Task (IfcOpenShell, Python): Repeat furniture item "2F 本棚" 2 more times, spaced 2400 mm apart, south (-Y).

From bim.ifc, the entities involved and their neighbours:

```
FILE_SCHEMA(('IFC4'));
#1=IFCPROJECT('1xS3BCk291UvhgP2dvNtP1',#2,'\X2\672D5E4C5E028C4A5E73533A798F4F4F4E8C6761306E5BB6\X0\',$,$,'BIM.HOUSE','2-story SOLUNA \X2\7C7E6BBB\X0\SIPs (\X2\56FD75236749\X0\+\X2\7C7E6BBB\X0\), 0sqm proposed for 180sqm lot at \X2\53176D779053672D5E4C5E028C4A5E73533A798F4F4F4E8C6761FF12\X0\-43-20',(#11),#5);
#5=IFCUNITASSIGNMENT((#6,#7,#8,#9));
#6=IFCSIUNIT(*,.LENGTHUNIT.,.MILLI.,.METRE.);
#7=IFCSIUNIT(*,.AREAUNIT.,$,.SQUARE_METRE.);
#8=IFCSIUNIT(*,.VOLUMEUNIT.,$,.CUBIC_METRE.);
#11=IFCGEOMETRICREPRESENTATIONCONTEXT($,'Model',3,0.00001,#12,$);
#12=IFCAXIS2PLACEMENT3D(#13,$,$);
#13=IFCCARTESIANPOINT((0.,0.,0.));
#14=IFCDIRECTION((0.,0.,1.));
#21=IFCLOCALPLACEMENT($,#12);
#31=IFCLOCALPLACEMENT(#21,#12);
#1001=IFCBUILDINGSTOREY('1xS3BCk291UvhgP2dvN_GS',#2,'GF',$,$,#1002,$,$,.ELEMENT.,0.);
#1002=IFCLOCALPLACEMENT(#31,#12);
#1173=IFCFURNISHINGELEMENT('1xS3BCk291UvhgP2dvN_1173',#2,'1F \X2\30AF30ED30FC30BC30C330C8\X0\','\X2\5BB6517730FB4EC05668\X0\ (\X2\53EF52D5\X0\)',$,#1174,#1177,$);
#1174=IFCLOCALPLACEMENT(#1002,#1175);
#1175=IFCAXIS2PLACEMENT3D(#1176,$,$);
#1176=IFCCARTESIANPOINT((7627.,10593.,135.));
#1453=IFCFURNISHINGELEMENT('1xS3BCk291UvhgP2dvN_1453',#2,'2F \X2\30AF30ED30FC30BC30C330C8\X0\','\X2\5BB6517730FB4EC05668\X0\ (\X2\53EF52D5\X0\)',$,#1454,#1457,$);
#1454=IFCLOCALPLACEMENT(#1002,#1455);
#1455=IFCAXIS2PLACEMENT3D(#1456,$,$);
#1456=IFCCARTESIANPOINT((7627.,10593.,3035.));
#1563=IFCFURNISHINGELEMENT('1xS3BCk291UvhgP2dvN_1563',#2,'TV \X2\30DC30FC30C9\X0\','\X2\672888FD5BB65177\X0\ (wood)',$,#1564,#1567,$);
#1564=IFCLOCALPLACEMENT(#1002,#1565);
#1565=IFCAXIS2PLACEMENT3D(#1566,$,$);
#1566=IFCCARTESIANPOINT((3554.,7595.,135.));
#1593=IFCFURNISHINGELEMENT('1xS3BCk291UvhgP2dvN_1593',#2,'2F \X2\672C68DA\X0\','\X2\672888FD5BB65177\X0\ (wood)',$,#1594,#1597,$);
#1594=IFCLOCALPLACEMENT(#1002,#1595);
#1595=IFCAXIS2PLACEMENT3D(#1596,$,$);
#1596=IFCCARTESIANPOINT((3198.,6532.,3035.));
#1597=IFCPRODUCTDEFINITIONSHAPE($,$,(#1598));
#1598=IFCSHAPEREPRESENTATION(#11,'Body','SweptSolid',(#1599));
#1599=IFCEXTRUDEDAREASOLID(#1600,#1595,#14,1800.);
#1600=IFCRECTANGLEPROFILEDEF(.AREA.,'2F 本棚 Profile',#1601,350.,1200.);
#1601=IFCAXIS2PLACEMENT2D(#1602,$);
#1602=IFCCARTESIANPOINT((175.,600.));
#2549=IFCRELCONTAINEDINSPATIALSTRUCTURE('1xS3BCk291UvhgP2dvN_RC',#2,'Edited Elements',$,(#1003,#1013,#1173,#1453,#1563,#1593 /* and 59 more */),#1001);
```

```python
import numpy as np
import ifcopenshell
import ifcopenshell.api.geometry
import ifcopenshell.api.root
import ifcopenshell.util.element
import ifcopenshell.util.placement

model = ifcopenshell.open("bim.ifc")


def reuse_history(source, copy):
    """copy_class also copies each property set's owner history, people and application; keep the originals."""
    for rel in copy.IsDefinedBy:
        if rel.is_a("IfcRelDefinesByProperties") and (history := rel.RelatingPropertyDefinition.OwnerHistory):
            rel.RelatingPropertyDefinition.OwnerHistory = source.OwnerHistory
            ifcopenshell.util.element.remove_deep2(model, history)


source = model.by_id(1593)
base = ifcopenshell.util.placement.get_local_placement(source.ObjectPlacement)
step = np.array([0.0, -1.0, 0.0]) * 2400.0

for i in range(1, 3):
    copy = ifcopenshell.api.root.copy_class(model, product=source)
    copy.Representation = ifcopenshell.util.element.copy_deep(
        model, source.Representation, exclude=["IfcGeometricRepresentationContext", "IfcRepresentationMap"]
    )
    reuse_history(source, copy)
    matrix = base.copy()
    matrix[:3, 3] += i * step
    print("added at", matrix[:3, 3].round(3) + 0.0)
    ifcopenshell.api.geometry.edit_object_placement(model, product=copy, matrix=matrix, is_si=False)

model.write("bim_rev.ifc")
```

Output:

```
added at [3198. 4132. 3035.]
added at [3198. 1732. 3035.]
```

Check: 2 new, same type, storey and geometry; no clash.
